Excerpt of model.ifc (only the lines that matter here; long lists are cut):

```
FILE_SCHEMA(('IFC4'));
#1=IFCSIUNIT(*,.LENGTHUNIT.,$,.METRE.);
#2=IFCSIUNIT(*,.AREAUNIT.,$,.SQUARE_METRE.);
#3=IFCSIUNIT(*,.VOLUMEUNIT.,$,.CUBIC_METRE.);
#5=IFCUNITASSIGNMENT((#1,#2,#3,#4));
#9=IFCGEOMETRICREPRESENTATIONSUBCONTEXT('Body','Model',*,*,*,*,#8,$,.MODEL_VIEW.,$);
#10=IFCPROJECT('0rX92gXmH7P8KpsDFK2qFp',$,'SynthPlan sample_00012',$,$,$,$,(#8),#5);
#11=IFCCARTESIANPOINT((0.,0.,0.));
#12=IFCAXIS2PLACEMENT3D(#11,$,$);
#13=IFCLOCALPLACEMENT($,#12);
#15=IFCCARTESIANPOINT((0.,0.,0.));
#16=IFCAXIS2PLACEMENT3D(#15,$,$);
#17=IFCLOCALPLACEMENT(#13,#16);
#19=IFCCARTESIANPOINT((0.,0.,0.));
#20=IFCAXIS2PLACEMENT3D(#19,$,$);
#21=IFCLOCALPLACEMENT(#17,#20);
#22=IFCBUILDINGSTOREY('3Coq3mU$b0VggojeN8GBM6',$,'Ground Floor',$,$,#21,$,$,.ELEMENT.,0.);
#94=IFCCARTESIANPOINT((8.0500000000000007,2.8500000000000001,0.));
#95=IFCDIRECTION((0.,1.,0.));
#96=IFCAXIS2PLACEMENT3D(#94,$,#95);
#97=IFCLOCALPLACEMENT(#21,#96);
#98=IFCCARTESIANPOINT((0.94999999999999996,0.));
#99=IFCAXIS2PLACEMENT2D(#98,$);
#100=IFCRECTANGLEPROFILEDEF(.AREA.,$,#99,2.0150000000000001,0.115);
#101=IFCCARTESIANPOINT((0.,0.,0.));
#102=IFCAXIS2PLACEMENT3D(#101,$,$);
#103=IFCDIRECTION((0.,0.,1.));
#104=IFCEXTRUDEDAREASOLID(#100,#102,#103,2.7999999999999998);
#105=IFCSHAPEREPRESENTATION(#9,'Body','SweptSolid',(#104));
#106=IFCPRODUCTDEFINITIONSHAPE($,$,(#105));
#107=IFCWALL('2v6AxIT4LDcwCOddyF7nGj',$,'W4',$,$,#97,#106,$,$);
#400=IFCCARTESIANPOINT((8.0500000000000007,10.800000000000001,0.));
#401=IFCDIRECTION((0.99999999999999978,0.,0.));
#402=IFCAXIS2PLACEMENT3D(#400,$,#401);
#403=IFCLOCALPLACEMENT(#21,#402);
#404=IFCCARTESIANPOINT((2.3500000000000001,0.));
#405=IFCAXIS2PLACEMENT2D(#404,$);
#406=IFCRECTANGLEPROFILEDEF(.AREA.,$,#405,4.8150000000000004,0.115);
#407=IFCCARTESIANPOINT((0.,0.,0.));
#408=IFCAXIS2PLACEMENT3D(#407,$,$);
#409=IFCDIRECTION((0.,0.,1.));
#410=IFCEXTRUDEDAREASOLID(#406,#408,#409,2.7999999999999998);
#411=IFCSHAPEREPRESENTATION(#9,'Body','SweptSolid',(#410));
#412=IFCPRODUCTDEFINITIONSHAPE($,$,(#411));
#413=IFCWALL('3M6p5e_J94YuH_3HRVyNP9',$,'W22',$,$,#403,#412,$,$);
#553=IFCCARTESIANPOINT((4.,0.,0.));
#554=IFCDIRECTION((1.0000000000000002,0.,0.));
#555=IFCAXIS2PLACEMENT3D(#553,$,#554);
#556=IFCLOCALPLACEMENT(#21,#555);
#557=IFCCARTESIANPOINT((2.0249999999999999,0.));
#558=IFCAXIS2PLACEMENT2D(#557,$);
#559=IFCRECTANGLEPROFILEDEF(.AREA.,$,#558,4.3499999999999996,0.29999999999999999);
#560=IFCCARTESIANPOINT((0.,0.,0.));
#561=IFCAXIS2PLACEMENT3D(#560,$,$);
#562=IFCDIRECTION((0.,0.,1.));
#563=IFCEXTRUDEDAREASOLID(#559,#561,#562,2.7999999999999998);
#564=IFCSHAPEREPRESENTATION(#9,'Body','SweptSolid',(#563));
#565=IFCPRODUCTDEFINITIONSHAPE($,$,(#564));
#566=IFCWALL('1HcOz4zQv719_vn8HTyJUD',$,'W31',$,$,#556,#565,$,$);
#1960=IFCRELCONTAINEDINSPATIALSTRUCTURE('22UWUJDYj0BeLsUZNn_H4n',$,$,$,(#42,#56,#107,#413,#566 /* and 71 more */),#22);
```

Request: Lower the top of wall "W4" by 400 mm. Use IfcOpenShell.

```python
import ifcopenshell
import ifcopenshell.geom
import ifcopenshell.util.representation
import ifcopenshell.util.shape
import ifcopenshell.util.unit

model = ifcopenshell.open("model.ifc")
unit_scale = ifcopenshell.util.unit.calculate_unit_scale(model)
settings = ifcopenshell.geom.settings()


def volume(element):
    """Net volume in cubic metres, openings subtracted."""
    shape = ifcopenshell.geom.create_shape(settings, element)
    return ifcopenshell.util.shape.get_volume(shape.geometry)


wall = model.by_guid("2v6AxIT4LDcwCOddyF7nGj")
before = volume(wall)

body = ifcopenshell.util.representation.get_representation(wall, "Model", "Body")
solid = body.Items[0]
old_height = solid.Depth
solid.Depth -= 0.4 / unit_scale
after = volume(wall)

print(f"height {old_height:g} -> {solid.Depth:g}, volume {before:.3f} -> {after:.3f} m3")

model.write("model-out.ifc")
```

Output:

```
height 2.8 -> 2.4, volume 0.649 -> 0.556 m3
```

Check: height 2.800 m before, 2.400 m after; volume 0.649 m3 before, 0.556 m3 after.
